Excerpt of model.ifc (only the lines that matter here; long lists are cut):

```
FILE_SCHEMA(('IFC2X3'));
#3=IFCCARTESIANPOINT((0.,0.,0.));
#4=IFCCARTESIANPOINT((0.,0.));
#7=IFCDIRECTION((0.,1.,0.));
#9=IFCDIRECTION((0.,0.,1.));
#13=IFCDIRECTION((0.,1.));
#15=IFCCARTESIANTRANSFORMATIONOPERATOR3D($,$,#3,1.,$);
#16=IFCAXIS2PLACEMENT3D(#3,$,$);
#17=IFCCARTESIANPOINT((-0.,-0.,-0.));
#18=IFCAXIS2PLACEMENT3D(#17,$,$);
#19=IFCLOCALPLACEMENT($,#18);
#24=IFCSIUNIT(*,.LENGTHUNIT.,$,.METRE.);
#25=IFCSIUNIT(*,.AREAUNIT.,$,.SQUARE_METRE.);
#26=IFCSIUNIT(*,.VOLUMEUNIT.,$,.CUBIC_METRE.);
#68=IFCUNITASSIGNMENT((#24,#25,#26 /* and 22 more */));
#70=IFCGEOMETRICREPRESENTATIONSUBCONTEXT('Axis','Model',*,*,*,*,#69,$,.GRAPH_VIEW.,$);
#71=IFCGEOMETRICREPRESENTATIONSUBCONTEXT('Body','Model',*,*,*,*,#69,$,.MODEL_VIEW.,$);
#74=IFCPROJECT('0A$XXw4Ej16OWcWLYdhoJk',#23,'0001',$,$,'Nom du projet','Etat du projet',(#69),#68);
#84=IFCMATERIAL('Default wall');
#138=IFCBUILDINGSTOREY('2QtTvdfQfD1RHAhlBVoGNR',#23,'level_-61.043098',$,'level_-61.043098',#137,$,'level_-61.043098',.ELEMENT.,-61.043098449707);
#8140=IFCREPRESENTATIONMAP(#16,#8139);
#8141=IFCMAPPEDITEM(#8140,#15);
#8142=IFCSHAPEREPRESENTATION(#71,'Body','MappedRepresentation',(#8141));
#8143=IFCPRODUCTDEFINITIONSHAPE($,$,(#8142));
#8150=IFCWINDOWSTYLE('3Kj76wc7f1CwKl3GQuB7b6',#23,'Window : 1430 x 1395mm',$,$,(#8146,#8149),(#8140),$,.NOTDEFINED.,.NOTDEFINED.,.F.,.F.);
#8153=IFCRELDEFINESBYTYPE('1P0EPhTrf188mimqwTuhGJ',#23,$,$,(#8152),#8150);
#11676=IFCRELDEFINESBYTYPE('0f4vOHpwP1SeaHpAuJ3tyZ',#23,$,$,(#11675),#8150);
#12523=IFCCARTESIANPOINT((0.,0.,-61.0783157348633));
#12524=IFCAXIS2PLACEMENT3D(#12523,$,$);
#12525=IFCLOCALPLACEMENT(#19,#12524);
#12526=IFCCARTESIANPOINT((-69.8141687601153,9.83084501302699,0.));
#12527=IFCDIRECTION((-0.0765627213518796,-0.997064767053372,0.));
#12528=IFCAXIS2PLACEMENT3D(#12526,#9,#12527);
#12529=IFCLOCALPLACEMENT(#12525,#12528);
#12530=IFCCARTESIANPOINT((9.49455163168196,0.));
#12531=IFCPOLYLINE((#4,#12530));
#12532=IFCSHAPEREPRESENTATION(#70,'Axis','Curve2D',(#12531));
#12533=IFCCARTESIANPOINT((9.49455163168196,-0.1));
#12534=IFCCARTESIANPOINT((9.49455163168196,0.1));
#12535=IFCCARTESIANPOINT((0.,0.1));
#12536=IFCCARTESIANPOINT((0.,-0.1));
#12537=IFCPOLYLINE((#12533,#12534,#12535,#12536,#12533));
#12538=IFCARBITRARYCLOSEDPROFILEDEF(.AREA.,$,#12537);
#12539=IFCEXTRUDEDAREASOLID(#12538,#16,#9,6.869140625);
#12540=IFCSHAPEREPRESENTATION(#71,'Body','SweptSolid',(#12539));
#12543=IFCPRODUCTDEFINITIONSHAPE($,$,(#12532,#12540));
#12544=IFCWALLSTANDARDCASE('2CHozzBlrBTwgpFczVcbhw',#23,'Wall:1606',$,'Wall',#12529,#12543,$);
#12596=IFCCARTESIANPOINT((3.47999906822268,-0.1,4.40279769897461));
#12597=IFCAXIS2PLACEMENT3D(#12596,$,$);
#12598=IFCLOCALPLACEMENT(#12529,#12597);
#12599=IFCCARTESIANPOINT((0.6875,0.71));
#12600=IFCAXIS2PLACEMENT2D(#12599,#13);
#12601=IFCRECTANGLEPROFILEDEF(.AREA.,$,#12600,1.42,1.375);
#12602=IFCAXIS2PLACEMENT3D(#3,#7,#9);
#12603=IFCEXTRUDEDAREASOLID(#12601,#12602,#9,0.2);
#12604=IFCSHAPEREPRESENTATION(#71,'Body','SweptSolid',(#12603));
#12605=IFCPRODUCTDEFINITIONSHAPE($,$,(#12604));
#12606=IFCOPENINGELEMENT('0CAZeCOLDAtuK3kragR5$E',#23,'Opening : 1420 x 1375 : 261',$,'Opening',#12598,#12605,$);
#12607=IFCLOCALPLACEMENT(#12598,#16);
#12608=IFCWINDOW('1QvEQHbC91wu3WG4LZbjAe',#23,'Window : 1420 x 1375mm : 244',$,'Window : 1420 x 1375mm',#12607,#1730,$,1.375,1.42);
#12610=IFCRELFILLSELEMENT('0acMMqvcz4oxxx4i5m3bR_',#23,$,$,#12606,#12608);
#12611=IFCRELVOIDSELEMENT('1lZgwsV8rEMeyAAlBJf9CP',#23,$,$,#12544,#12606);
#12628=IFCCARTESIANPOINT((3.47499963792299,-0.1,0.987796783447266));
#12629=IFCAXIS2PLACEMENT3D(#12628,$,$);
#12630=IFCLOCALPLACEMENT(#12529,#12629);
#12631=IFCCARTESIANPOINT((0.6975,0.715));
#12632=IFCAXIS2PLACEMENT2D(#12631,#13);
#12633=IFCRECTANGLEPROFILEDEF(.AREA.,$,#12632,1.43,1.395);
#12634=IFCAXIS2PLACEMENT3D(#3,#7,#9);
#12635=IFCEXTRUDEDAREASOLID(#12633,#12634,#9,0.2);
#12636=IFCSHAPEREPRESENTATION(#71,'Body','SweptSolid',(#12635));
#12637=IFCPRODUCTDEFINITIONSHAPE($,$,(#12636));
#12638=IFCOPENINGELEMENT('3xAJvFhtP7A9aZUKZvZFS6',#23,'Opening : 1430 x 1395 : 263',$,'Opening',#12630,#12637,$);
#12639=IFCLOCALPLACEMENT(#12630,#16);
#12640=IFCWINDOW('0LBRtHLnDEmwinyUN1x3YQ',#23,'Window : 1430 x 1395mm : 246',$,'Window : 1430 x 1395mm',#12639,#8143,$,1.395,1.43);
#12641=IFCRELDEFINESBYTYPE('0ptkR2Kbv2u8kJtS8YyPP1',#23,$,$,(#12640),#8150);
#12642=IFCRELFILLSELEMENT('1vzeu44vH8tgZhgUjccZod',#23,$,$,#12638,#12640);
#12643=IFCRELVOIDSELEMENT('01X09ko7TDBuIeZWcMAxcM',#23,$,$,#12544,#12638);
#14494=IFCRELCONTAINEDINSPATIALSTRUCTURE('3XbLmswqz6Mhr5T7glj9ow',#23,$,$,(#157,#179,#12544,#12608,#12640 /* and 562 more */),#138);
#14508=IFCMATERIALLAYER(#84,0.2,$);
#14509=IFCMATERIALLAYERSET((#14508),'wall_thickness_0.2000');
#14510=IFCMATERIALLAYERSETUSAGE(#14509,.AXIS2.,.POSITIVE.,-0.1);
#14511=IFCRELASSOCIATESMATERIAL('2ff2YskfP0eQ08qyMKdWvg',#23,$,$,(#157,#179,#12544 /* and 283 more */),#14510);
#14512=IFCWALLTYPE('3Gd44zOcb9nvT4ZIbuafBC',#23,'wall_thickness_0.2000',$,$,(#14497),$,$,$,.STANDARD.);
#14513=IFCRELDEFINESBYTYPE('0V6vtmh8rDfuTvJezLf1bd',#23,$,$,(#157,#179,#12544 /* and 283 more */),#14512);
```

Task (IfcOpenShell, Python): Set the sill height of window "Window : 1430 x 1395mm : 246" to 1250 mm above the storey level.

```python
import numpy as np
import ifcopenshell
import ifcopenshell.api.geometry
import ifcopenshell.geom
import ifcopenshell.util.element
import ifcopenshell.util.placement
import ifcopenshell.util.shape
import ifcopenshell.util.unit

model = ifcopenshell.open("model.ifc")
unit_scale = ifcopenshell.util.unit.calculate_unit_scale(model)

window = model.by_guid("0LBRtHLnDEmwinyUN1x3YQ")
opening = window.FillsVoids[0].RelatingOpeningElement
storey = ifcopenshell.util.element.get_container(window, ifc_class="IfcBuildingStorey")
level = ifcopenshell.util.placement.get_local_placement(storey.ObjectPlacement)[2, 3]

# The opening's origin need not be at the sill, so measure its lowest point.
shape = ifcopenshell.geom.create_shape(ifcopenshell.geom.settings(), opening)
bottom = ifcopenshell.util.shape.get_shape_bottom_elevation(shape, shape.geometry) / unit_scale
dz = level + 1.25 - bottom

shift = np.array([0.0, 0.0, dz])
# The window is placed relative to its opening, so it follows when the opening moves.
matrix = ifcopenshell.util.placement.get_local_placement(opening.ObjectPlacement)
matrix[:3, 3] += shift
ifcopenshell.api.geometry.edit_object_placement(
    model, product=opening, matrix=matrix, is_si=False, should_transform_children=True
)

print(f"moved by {dz * unit_scale:+.3f} m")

model.write("model_edited.ifc")
```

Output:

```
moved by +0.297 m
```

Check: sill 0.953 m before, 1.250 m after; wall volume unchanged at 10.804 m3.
